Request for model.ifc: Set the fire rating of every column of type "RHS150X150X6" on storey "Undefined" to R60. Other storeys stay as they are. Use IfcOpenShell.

First a look at what the model holds.

```python
import ifcopenshell
import ifcopenshell.util.element

model = ifcopenshell.open("model.ifc")
print(model.schema)
storey = next(s for s in model.by_type("IfcBuildingStorey") if s.Name == "Undefined")
columns = [e for e in ifcopenshell.util.element.get_decomposition(storey) if e.is_a("IfcColumn")]
seen = {}
for e in columns:
    element_type = ifcopenshell.util.element.get_type(e)
    key = (element_type.Name if element_type != e and element_type else None, ifcopenshell.util.element.get_pset(e, "Pset_ColumnCommon", "FireRating"))
    seen[key] = seen.get(key, 0) + 1
for (name, value), count in sorted(seen.items(), key=str):
    print(count, "x", name, "|", value)
```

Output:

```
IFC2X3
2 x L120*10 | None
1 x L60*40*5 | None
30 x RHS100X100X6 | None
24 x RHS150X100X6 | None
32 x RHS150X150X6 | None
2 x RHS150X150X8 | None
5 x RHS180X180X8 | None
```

```python
import ifcopenshell
import ifcopenshell.api.pset
import ifcopenshell.util.element

model = ifcopenshell.open("model.ifc")

storey = next(s for s in model.by_type("IfcBuildingStorey") if s.Name == "Undefined")
columns = [e for e in ifcopenshell.util.element.get_decomposition(storey) if e.is_a("IfcColumn")]

count = 0
for e in columns:
    element_type = ifcopenshell.util.element.get_type(e)
    if element_type in (None, e) or element_type.Name != "RHS150X150X6":
        continue
    found = ifcopenshell.util.element.get_pset(e, "Pset_ColumnCommon", should_inherit=False)
    if found:
        pset = model.by_id(found["id"])
        if len(ifcopenshell.util.element.get_elements_by_pset(pset)) > 1:
            pset = ifcopenshell.api.pset.unshare_pset(model, products=[e], pset=pset)[0]
    else:
        pset = ifcopenshell.api.pset.add_pset(model, product=e, name="Pset_ColumnCommon")
    ifcopenshell.api.pset.edit_pset(model, pset=pset, properties={"FireRating": "R60"})
    count += 1

print(count, "columns updated")

model.write("model-out.ifc")
```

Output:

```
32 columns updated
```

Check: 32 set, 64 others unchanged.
